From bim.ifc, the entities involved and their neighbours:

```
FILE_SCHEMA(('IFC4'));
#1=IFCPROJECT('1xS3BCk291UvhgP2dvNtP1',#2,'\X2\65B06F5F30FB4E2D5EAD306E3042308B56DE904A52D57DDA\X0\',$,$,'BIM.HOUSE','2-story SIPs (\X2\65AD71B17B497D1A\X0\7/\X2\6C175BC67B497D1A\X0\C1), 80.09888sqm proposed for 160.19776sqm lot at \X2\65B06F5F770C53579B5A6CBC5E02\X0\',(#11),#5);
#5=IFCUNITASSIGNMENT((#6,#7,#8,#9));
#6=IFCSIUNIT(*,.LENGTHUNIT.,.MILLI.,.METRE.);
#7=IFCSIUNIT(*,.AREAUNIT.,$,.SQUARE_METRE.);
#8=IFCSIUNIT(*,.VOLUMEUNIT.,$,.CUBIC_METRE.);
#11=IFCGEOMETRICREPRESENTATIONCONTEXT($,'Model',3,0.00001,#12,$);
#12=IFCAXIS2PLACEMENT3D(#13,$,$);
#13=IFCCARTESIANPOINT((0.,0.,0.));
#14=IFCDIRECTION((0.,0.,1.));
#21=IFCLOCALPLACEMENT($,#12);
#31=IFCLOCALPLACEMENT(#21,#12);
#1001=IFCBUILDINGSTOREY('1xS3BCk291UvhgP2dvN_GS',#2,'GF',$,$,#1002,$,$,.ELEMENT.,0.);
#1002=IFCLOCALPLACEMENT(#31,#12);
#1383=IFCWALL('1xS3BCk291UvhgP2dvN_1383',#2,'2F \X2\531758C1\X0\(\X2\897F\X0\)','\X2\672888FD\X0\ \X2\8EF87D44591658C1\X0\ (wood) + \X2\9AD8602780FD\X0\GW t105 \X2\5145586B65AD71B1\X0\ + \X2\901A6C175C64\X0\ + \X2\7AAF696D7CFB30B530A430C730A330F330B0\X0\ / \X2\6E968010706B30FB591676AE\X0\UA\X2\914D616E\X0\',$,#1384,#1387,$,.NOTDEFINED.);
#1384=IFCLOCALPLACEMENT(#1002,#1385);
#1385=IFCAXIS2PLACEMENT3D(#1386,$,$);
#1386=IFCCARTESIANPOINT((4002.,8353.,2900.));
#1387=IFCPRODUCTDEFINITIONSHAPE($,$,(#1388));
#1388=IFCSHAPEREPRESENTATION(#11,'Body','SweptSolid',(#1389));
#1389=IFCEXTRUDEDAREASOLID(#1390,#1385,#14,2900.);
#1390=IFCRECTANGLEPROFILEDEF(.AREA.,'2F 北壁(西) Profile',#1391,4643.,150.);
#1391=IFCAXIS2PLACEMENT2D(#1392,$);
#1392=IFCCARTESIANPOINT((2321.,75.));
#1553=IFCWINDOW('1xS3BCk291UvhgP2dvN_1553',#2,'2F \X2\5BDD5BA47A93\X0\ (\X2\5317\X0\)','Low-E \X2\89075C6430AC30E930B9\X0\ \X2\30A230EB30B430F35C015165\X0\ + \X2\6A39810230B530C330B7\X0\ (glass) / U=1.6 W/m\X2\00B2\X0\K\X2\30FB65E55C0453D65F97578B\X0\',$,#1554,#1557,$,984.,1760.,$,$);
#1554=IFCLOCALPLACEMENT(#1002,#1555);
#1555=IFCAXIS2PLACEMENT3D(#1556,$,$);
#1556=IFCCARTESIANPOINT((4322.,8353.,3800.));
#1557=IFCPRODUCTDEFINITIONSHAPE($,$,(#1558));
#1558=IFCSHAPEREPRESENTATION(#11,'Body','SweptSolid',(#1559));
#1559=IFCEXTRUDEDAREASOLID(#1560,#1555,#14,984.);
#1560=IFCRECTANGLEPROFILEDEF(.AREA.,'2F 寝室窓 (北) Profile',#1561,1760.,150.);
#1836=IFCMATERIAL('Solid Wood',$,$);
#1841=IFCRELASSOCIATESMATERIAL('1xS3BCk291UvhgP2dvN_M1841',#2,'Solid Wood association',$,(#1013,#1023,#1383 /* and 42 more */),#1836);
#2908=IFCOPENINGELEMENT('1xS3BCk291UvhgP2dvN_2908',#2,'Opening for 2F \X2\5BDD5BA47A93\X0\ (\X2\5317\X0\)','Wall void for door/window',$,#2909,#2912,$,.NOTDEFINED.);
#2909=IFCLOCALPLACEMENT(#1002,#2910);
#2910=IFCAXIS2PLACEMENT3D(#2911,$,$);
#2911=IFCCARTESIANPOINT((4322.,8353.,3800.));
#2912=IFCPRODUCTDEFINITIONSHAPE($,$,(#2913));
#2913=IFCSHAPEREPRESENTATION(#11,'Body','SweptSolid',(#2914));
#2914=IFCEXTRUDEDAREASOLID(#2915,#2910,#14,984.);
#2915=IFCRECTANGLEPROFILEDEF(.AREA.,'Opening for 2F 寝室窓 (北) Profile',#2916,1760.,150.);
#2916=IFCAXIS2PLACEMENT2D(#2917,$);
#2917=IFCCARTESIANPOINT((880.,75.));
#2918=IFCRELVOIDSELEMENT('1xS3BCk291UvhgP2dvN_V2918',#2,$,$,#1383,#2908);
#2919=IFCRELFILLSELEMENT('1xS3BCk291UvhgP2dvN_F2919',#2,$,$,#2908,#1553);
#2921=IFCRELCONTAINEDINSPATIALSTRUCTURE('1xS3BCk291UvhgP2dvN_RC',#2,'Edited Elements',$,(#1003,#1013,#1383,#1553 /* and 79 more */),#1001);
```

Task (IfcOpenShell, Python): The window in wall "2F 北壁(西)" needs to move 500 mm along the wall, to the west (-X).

```python
import ifcopenshell
import ifcopenshell.api.geometry
import ifcopenshell.util.placement
import ifcopenshell.util.unit

model = ifcopenshell.open("bim.ifc")
unit_scale = ifcopenshell.util.unit.calculate_unit_scale(model)

window = model.by_guid("1xS3BCk291UvhgP2dvN_1553")
opening = window.FillsVoids[0].RelatingOpeningElement
wall = opening.VoidsElements[0].RelatingBuildingElement

wall_matrix = ifcopenshell.util.placement.get_local_placement(wall.ObjectPlacement)
shift = wall_matrix[:3, 0] * -0.5 / unit_scale
before = ifcopenshell.util.placement.get_local_placement(window.ObjectPlacement)[:3, 3].copy()

# The window is not placed relative to its opening, so move both.
for product in (opening, window):
    matrix = ifcopenshell.util.placement.get_local_placement(product.ObjectPlacement)
    matrix[:3, 3] += shift
    ifcopenshell.api.geometry.edit_object_placement(model, product=product, matrix=matrix, is_si=False)

after = ifcopenshell.util.placement.get_local_placement(window.ObjectPlacement)[:3, 3]
print("window moved by", (after - before).round(3) + 0.0)

model.write("bim_edited.ifc")
```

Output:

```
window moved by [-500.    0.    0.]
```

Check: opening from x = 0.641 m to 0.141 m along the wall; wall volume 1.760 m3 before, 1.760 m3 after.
